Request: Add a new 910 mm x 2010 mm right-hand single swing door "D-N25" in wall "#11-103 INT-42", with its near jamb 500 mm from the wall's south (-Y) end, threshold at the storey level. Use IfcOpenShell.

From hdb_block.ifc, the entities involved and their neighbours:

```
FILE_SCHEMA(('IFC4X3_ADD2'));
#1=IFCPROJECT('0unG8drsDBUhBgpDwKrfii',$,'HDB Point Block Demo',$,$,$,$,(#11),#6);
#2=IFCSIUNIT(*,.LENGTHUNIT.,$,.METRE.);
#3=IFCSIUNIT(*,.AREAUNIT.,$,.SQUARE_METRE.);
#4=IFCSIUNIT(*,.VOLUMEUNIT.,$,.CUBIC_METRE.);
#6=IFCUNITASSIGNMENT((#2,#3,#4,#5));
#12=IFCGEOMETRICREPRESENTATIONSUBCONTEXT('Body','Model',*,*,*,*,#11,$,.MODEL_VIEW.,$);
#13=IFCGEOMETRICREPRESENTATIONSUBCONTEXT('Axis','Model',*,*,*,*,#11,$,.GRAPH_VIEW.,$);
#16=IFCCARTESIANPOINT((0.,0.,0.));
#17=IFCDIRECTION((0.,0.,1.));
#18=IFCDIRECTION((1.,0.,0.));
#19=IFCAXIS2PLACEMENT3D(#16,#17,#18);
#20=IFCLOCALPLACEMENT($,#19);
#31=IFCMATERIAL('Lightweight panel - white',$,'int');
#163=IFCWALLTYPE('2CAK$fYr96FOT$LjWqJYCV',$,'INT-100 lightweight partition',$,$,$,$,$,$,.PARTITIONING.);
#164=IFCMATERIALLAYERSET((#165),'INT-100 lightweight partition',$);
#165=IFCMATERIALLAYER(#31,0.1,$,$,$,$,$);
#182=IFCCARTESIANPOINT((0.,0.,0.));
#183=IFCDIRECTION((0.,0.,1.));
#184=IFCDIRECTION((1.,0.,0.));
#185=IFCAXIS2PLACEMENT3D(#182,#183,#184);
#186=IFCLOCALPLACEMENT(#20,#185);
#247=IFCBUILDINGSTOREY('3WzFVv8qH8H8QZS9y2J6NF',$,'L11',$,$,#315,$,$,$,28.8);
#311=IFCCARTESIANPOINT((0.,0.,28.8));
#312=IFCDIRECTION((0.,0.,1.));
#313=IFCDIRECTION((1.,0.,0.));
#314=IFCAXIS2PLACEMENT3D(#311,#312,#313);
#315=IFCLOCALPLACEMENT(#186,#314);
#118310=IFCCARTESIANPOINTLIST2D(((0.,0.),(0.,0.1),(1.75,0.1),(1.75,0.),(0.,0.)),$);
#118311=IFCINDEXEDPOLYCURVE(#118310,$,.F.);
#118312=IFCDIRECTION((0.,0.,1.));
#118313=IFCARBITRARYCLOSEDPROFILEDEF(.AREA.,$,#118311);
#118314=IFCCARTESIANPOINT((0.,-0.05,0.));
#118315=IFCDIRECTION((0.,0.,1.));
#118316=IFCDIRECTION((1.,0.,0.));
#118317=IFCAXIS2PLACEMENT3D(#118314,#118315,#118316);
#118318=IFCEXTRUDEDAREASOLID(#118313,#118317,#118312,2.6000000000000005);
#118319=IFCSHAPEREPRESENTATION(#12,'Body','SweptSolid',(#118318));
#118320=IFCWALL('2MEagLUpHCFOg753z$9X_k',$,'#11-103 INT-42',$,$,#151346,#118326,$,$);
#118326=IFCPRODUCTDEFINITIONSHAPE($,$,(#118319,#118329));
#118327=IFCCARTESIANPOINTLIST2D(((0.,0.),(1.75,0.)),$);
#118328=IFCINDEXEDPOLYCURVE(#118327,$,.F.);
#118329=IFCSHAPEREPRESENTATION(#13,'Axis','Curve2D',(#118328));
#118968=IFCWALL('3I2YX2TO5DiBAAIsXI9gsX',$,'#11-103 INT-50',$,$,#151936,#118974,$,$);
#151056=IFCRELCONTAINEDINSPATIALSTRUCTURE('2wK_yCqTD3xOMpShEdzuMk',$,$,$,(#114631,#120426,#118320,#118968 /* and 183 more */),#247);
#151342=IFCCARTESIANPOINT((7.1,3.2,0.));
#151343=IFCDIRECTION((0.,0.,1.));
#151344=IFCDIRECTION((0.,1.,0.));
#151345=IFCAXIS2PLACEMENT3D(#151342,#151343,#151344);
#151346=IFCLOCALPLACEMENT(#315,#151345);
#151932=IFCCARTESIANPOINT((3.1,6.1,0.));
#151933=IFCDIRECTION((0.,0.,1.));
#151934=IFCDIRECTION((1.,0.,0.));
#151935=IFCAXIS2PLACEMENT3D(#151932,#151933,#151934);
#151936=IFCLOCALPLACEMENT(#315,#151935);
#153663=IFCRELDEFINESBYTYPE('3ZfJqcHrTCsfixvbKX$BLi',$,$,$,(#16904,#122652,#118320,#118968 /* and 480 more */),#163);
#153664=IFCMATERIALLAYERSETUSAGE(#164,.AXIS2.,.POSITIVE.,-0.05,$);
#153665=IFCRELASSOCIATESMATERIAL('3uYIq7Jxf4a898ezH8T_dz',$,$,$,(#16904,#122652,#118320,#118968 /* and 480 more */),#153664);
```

```python
import numpy as np
import ifcopenshell
import ifcopenshell.api.feature
import ifcopenshell.api.geometry
import ifcopenshell.api.root
import ifcopenshell.api.spatial
import ifcopenshell.geom
import ifcopenshell.util.element
import ifcopenshell.util.placement
import ifcopenshell.util.representation
import ifcopenshell.util.shape
import ifcopenshell.util.unit

model = ifcopenshell.open("hdb_block.ifc")
unit_scale = ifcopenshell.util.unit.calculate_unit_scale(model)
settings = ifcopenshell.geom.settings()


def volume(element):
    """Net volume in cubic metres, openings subtracted."""
    shape = ifcopenshell.geom.create_shape(settings, element)
    return ifcopenshell.util.shape.get_volume(shape.geometry)


wall = model.by_guid("2MEagLUpHCFOg753z$9X_k")
storey = ifcopenshell.util.element.get_container(wall, ifc_class="IfcBuildingStorey")
context = ifcopenshell.util.representation.get_context(model, "Model", "Body", "MODEL_VIEW")
before = volume(wall)

width, height, from_end, sill = 0.91, 2.01, 0.5, 0.0  # metres

# The wall runs along its own X axis, and the end named is its -X end.
wall_shape = ifcopenshell.geom.create_shape(settings, wall)
x, y, z = ifcopenshell.util.shape.get_vertices(wall_shape.geometry).T
start = x.min() + from_end
face, thickness = float(y.min()), float(y.max() - y.min())
wall_matrix = ifcopenshell.util.placement.get_local_placement(wall.ObjectPlacement)
level = ifcopenshell.util.placement.get_local_placement(storey.ObjectPlacement)[2, 3]


def in_wall(x, y):
    """Placement at x, y metres in the wall's axes, at sill height."""
    matrix = wall_matrix.copy()
    matrix[:, 3] = wall_matrix @ np.array([x / unit_scale, y / unit_scale, 0.0, 1.0])
    matrix[2, 3] = level + sill / unit_scale
    return matrix


# Opening: a box that overshoots both wall faces by 50 mm.
opening = ifcopenshell.api.root.create_entity(model, ifc_class="IfcOpeningElement", predefined_type="OPENING")
box = ifcopenshell.api.geometry.add_wall_representation(
    model, context=context, length=width, height=height, thickness=thickness + 0.1
)
ifcopenshell.api.geometry.assign_representation(model, product=opening, representation=box)
ifcopenshell.api.geometry.edit_object_placement(model, product=opening, matrix=in_wall(start, face - 0.05), is_si=False)
ifcopenshell.api.feature.add_feature(model, feature=opening, element=wall)

door = ifcopenshell.api.root.create_entity(model, ifc_class="IfcDoor", name="D-N25", predefined_type="DOOR")
door.OverallWidth, door.OverallHeight = width / unit_scale, height / unit_scale
door.OperationType = "SINGLE_SWING_RIGHT"
body = ifcopenshell.api.geometry.add_door_representation(
    model,
    context=context,
    overall_width=door.OverallWidth,
    overall_height=door.OverallHeight,
    operation_type="SINGLE_SWING_RIGHT",
    lining_properties={"LiningDepth": thickness / unit_scale, "ThresholdDepth": thickness / unit_scale},
)
ifcopenshell.api.geometry.assign_representation(model, product=door, representation=body)
ifcopenshell.api.spatial.assign_container(model, products=[door], relating_structure=storey)
ifcopenshell.api.feature.add_filling(model, opening=opening, element=door)

# The lining spans the wall, so the door starts at the wall face.
ifcopenshell.api.geometry.edit_object_placement(model, product=door, matrix=in_wall(start, face), is_si=False)

after = volume(wall)

print(f"wall volume {before:.3f} -> {after:.3f} m3")

model.write("hdb_block_v2.ifc")
```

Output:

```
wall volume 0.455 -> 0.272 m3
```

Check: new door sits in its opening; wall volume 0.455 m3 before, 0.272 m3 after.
